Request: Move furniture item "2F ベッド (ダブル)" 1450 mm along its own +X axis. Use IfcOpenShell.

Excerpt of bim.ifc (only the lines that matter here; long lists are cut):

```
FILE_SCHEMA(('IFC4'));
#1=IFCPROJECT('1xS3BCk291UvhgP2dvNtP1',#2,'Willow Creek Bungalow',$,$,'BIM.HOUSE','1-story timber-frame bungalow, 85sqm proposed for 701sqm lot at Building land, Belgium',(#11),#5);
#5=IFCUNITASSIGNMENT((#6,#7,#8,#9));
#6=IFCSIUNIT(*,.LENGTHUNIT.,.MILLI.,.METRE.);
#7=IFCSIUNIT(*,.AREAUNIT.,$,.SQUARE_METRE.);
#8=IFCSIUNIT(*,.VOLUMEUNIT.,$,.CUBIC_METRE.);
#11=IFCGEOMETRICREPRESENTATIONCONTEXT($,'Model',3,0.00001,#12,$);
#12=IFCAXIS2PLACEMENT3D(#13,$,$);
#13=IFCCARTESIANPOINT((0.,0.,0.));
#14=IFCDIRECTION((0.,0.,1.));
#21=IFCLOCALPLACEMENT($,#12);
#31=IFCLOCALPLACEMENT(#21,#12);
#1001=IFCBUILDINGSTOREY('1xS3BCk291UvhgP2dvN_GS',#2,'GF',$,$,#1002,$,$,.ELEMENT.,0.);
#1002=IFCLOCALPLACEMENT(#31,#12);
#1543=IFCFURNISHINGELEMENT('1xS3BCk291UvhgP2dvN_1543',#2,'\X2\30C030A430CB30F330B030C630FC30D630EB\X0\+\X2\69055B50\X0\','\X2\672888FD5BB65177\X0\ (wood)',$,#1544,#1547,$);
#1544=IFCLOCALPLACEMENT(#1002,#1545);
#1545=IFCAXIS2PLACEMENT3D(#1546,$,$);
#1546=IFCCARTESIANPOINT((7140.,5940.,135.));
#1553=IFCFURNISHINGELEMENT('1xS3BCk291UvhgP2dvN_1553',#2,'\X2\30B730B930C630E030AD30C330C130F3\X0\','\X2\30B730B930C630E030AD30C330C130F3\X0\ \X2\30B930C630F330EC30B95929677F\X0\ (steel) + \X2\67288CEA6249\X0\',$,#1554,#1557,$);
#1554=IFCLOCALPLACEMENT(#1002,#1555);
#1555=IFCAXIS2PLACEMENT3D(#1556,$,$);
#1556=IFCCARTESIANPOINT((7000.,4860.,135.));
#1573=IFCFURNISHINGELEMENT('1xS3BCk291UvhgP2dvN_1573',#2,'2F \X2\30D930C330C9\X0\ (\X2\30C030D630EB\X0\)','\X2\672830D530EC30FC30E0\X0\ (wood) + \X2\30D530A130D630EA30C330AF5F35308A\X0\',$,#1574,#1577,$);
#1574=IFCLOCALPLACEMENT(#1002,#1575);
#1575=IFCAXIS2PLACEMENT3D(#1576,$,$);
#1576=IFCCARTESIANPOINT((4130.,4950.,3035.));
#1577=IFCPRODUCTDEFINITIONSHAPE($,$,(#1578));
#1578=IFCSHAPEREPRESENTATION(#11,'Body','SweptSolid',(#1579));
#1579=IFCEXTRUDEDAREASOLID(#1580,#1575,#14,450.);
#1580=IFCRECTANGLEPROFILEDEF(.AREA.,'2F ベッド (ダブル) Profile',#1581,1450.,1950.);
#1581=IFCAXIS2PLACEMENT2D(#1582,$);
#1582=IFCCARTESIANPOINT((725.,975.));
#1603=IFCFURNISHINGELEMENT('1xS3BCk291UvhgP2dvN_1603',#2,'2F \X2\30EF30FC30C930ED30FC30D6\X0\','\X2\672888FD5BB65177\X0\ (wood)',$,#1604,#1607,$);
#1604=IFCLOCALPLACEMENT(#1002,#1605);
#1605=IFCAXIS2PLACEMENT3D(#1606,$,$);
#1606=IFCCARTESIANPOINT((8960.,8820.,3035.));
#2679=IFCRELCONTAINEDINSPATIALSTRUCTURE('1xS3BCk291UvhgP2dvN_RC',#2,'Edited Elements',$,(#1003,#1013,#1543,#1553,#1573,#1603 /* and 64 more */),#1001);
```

```python
import ifcopenshell
import ifcopenshell.api.geometry
import ifcopenshell.util.placement

model = ifcopenshell.open("bim.ifc")

item = model.by_guid("1xS3BCk291UvhgP2dvN_1573")
matrix = ifcopenshell.util.placement.get_local_placement(item.ObjectPlacement)
matrix[:3, 3] += matrix[:3, 0] * 1450.0
ifcopenshell.api.geometry.edit_object_placement(model, product=item, matrix=matrix, is_si=False)

print(ifcopenshell.util.placement.get_local_placement(item.ObjectPlacement).round(3) + 0.0)

model.write("bim-out.ifc")
```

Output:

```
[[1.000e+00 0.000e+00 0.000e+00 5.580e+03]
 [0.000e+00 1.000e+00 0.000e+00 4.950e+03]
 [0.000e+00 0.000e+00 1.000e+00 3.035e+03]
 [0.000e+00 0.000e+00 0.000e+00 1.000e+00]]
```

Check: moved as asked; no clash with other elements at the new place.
